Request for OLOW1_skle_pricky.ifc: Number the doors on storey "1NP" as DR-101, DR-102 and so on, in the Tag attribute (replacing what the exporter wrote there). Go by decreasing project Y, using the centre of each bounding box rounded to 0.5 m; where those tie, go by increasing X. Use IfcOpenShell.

First a look at what the model holds.

```python
import ifcopenshell
import ifcopenshell.util.element
import ifcopenshell.util.placement

model = ifcopenshell.open("OLOW1_skle_pricky.ifc")
print(model.schema)
storey = next(s for s in model.by_type("IfcBuildingStorey") if s.Name == "1NP")
doors = [e for e in ifcopenshell.util.element.get_decomposition(storey) if e.is_a("IfcDoor")]
for e in sorted(doors, key=lambda e: e.id()):
    origin = ifcopenshell.util.placement.get_local_placement(e.ObjectPlacement)[:3, 3]
    print(e.id(), e.Tag, e.Name, origin.round(2) + 0.0, sep=" | ")
```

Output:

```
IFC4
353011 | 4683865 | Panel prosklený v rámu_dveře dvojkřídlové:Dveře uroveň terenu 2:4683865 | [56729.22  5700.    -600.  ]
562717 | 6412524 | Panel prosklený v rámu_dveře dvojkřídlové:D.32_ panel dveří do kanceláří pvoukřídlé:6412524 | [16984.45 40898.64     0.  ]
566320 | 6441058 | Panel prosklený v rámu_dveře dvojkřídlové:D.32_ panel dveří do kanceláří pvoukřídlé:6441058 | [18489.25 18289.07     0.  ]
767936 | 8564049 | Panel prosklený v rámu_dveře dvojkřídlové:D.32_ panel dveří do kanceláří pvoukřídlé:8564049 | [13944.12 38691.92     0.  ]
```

```python
import ifcopenshell
import ifcopenshell.geom
import ifcopenshell.util.element
import ifcopenshell.util.shape

model = ifcopenshell.open("OLOW1_skle_pricky.ifc")
settings = ifcopenshell.geom.settings()
settings.set("use-world-coords", True)


def centre(element):
    shape = ifcopenshell.geom.create_shape(settings, element)
    return ifcopenshell.util.shape.get_bbox_centroid(shape.geometry)


storey = next(s for s in model.by_type("IfcBuildingStorey") if s.Name == "1NP")
doors = [e for e in ifcopenshell.util.element.get_decomposition(storey) if e.is_a("IfcDoor")]

# Insertion points can sit at a corner or the storey origin, so sort by the geometry (in metres).
centres = {e: centre(e) for e in doors}
doors.sort(key=lambda e: (-round(centres[e][1] / 0.5), centres[e][0]))

for i, e in enumerate(doors, start=1):
    number = f"DR-1{i:02d}"
    e.Tag = number
    print(e.id(), number)

model.write("OLOW1_skle_pricky_updated.ifc")
```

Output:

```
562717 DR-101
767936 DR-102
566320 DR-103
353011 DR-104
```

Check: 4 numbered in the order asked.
